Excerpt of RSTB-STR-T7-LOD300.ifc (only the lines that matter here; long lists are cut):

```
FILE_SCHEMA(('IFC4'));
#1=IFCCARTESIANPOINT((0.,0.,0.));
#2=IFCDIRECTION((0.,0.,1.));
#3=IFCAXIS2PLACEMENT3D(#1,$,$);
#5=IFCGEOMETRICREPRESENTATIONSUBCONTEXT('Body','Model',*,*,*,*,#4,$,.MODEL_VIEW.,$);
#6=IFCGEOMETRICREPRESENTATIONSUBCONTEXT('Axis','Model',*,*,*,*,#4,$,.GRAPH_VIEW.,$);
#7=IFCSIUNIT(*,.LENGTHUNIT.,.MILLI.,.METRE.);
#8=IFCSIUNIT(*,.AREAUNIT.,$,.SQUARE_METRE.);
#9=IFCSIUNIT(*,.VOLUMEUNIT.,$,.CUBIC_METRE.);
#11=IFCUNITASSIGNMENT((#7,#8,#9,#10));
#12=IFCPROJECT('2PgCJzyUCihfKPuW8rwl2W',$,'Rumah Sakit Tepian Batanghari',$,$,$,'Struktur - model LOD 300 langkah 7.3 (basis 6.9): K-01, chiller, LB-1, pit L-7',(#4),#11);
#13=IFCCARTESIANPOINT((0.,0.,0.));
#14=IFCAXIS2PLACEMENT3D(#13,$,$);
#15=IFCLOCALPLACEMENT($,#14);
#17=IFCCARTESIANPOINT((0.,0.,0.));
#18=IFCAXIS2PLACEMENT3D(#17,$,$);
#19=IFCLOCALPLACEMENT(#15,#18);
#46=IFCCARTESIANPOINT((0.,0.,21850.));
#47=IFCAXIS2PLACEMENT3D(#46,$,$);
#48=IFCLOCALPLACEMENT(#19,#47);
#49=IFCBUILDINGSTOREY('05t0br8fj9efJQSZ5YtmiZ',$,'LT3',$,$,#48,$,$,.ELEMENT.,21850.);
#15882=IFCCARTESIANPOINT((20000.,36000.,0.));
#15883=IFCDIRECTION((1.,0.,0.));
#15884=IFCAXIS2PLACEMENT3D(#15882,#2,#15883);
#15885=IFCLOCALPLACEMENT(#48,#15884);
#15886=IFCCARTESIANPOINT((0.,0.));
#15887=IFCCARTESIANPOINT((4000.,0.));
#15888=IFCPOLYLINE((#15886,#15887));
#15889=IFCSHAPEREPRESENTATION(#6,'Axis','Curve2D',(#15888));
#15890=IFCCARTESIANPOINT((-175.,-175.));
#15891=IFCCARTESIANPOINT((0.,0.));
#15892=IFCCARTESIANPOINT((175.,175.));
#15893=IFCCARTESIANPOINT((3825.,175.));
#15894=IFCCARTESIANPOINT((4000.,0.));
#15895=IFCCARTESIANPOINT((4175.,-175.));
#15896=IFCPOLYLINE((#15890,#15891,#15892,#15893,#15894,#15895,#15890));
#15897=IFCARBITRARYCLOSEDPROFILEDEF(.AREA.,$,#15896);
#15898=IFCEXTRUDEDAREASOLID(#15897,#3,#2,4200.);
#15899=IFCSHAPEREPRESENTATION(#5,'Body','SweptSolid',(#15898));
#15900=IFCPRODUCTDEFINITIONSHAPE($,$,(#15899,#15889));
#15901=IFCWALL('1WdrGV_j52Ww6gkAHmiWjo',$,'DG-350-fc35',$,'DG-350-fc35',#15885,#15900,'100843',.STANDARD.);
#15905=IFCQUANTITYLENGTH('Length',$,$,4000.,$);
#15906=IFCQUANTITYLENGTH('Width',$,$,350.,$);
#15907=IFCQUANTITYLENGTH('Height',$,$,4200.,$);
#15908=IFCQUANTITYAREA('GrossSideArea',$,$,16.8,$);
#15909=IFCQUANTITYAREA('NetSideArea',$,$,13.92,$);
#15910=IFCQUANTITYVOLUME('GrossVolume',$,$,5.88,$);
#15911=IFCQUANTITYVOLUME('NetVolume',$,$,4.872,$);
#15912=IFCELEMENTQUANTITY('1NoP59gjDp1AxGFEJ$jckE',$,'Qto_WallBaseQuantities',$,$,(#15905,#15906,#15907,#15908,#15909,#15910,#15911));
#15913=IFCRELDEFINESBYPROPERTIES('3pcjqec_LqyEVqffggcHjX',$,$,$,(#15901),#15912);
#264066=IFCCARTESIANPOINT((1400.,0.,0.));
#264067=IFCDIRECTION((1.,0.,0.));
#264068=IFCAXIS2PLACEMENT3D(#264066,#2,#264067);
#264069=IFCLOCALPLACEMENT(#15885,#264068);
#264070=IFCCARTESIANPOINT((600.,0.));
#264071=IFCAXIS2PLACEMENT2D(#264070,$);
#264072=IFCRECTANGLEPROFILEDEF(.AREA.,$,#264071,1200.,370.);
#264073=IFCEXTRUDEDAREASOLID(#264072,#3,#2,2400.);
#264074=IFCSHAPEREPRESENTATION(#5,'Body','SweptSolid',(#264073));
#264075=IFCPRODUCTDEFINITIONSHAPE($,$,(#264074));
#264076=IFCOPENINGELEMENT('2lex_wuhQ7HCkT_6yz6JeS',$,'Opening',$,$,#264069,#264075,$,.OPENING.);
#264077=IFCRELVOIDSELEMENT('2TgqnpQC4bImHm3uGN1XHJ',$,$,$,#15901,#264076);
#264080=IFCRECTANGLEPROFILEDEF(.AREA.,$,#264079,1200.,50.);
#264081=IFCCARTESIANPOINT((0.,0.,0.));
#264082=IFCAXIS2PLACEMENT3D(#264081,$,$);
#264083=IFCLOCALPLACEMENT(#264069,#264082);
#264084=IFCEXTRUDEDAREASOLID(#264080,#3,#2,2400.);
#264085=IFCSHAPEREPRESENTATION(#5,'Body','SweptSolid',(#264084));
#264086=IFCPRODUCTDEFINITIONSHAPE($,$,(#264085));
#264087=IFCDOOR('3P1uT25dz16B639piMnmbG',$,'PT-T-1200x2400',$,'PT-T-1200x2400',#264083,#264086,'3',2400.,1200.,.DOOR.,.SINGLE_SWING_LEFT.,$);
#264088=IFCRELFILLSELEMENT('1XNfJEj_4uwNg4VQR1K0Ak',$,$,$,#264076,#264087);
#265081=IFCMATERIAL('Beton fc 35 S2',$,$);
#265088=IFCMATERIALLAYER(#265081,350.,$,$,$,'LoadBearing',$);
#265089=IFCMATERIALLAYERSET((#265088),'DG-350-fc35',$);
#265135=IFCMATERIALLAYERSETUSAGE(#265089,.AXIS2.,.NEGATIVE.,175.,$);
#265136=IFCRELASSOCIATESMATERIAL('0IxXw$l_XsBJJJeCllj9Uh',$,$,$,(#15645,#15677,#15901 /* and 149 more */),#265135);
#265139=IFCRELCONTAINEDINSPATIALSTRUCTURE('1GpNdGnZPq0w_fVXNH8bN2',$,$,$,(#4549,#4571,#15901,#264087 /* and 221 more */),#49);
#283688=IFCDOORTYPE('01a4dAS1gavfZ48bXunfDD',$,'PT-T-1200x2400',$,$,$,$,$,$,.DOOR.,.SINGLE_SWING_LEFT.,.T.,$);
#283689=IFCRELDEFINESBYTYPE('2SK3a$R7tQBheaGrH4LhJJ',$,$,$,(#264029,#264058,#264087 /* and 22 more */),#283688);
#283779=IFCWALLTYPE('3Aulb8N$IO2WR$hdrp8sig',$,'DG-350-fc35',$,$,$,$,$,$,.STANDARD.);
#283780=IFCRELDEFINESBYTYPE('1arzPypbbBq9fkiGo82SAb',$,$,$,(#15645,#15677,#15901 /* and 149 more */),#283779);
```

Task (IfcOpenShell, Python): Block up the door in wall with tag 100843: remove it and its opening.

```python
import ifcopenshell
import ifcopenshell.api.feature
import ifcopenshell.api.pset
import ifcopenshell.api.root
import ifcopenshell.geom
import ifcopenshell.util.element
import ifcopenshell.util.shape
import ifcopenshell.util.unit

model = ifcopenshell.open("RSTB-STR-T7-LOD300.ifc")
area_scale = ifcopenshell.util.unit.calculate_unit_scale(model, "AREAUNIT")
volume_scale = ifcopenshell.util.unit.calculate_unit_scale(model, "VOLUMEUNIT")
settings = ifcopenshell.geom.settings()


def volume(element):
    """Net volume in cubic metres, openings subtracted."""
    shape = ifcopenshell.geom.create_shape(settings, element)
    return ifcopenshell.util.shape.get_volume(shape.geometry)


door = model.by_guid("3P1uT25dz16B639piMnmbG")
opening = door.FillsVoids[0].RelatingOpeningElement
wall = opening.VoidsElements[0].RelatingBuildingElement
before = volume(wall)

ifcopenshell.api.root.remove_product(model, product=door)
ifcopenshell.api.feature.remove_feature(model, feature=opening)

after = volume(wall)
thickness = 0.35  # wall thickness in metres

# Update the wall's stored quantities.
qto = model.by_id(ifcopenshell.util.element.get_pset(wall, "Qto_WallBaseQuantities", should_inherit=False)["id"])
ifcopenshell.api.pset.edit_qto(model, qto=qto, properties={
    "NetSideArea": after / thickness / area_scale,
    "NetVolume": after / volume_scale,
})

print(f"wall volume {before:.3f} -> {after:.3f} m3")

model.write("RSTB-STR-T7-LOD300_rev.ifc")
```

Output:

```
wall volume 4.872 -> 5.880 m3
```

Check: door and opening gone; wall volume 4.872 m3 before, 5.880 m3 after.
